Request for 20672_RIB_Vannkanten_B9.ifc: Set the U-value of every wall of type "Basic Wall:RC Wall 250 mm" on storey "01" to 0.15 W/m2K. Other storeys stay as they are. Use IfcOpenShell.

First a look at what the model holds.

```python
import ifcopenshell
import ifcopenshell.util.element

model = ifcopenshell.open("20672_RIB_Vannkanten_B9.ifc")
print(model.schema)
storey = next(s for s in model.by_type("IfcBuildingStorey") if s.Name == "01")
walls = [e for e in ifcopenshell.util.element.get_decomposition(storey) if e.is_a("IfcWall")]
seen = {}
for e in walls:
    element_type = ifcopenshell.util.element.get_type(e)
    key = (element_type.Name if element_type != e and element_type else None, ifcopenshell.util.element.get_pset(e, "Pset_WallCommon", "ThermalTransmittance"))
    seen[key] = seen.get(key, 0) + 1
for (name, value), count in sorted(seen.items(), key=str):
    print(count, "x", name, "|", value)
```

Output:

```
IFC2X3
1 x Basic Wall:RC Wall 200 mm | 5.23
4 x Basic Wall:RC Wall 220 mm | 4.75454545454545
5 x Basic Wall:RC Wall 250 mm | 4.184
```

```python
import ifcopenshell
import ifcopenshell.api.pset
import ifcopenshell.util.element

model = ifcopenshell.open("20672_RIB_Vannkanten_B9.ifc")

storey = next(s for s in model.by_type("IfcBuildingStorey") if s.Name == "01")
walls = [e for e in ifcopenshell.util.element.get_decomposition(storey) if e.is_a("IfcWall")]

count = 0
for e in walls:
    element_type = ifcopenshell.util.element.get_type(e)
    if element_type in (None, e) or element_type.Name != "Basic Wall:RC Wall 250 mm":
        continue
    # add_pset returns the element's existing set when there is one.
    pset = ifcopenshell.api.pset.add_pset(model, product=e, name="Pset_WallCommon")
    ifcopenshell.api.pset.edit_pset(model, pset=pset, properties={"ThermalTransmittance": 0.15})
    count += 1

print(count, "walls updated")

model.write("20672_RIB_Vannkanten_B9_rev.ifc")
```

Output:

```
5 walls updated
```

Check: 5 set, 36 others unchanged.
